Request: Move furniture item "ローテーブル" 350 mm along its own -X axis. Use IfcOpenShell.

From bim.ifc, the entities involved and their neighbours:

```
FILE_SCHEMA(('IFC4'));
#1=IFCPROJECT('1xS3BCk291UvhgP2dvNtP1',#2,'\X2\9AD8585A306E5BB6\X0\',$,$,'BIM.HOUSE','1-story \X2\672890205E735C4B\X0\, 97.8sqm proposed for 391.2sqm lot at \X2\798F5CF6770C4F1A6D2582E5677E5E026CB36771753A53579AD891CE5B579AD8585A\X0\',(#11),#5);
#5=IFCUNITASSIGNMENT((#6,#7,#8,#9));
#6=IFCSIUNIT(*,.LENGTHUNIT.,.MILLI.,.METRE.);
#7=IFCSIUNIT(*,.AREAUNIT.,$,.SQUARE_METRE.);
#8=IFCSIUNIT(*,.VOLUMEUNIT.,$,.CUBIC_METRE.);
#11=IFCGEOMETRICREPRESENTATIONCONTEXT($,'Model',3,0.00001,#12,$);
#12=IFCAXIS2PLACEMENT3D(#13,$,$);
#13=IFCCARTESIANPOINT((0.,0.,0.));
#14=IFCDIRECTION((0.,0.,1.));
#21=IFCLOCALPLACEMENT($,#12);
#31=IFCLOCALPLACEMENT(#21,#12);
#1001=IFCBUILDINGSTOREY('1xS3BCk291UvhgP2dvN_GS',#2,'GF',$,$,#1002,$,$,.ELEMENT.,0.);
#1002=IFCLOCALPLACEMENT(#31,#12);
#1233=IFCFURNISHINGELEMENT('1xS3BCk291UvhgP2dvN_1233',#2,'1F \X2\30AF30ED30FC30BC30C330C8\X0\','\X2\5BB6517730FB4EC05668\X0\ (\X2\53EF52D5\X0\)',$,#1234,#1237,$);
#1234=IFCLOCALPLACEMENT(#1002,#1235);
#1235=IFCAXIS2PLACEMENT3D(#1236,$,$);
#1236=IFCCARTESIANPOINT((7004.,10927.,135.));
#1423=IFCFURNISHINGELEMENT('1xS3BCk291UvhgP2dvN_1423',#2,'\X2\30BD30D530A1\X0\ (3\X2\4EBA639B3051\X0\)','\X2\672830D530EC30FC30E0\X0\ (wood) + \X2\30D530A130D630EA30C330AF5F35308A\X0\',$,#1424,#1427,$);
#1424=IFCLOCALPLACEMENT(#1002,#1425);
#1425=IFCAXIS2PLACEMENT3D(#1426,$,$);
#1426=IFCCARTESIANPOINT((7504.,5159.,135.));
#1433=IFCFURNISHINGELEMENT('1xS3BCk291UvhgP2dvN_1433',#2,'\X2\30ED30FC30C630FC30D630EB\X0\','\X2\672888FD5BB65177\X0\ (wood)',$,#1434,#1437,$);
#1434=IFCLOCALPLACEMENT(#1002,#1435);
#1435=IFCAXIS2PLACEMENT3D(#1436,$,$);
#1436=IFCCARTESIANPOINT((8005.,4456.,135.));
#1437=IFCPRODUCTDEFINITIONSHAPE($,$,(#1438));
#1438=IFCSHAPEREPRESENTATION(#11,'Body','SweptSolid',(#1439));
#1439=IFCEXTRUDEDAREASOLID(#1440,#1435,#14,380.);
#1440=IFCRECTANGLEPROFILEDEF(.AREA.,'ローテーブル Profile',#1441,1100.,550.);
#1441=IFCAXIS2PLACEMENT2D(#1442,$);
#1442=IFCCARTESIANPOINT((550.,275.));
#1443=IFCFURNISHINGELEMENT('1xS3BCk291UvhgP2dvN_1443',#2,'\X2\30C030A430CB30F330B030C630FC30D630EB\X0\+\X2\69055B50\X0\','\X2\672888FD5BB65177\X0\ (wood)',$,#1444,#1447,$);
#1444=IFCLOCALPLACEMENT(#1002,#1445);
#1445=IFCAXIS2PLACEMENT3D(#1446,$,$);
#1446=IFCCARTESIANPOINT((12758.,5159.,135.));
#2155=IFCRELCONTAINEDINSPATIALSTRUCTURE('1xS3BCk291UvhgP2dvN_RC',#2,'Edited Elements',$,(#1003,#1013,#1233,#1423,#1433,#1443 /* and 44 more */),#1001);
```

```python
import ifcopenshell
import ifcopenshell.api.geometry
import ifcopenshell.util.placement
import ifcopenshell.util.unit

model = ifcopenshell.open("bim.ifc")
unit_scale = ifcopenshell.util.unit.calculate_unit_scale(model)

item = model.by_guid("1xS3BCk291UvhgP2dvN_1433")
matrix = ifcopenshell.util.placement.get_local_placement(item.ObjectPlacement)
matrix[:3, 3] -= matrix[:3, 0] * 0.35 / unit_scale
ifcopenshell.api.geometry.edit_object_placement(model, product=item, matrix=matrix, is_si=False)

print(ifcopenshell.util.placement.get_local_placement(item.ObjectPlacement).round(3) + 0.0)

model.write("bim_v2.ifc")
```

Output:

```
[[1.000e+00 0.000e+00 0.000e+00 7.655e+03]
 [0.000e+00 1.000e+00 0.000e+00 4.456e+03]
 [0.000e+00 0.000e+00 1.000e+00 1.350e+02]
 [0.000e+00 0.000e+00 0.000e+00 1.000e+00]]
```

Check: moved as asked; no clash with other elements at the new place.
